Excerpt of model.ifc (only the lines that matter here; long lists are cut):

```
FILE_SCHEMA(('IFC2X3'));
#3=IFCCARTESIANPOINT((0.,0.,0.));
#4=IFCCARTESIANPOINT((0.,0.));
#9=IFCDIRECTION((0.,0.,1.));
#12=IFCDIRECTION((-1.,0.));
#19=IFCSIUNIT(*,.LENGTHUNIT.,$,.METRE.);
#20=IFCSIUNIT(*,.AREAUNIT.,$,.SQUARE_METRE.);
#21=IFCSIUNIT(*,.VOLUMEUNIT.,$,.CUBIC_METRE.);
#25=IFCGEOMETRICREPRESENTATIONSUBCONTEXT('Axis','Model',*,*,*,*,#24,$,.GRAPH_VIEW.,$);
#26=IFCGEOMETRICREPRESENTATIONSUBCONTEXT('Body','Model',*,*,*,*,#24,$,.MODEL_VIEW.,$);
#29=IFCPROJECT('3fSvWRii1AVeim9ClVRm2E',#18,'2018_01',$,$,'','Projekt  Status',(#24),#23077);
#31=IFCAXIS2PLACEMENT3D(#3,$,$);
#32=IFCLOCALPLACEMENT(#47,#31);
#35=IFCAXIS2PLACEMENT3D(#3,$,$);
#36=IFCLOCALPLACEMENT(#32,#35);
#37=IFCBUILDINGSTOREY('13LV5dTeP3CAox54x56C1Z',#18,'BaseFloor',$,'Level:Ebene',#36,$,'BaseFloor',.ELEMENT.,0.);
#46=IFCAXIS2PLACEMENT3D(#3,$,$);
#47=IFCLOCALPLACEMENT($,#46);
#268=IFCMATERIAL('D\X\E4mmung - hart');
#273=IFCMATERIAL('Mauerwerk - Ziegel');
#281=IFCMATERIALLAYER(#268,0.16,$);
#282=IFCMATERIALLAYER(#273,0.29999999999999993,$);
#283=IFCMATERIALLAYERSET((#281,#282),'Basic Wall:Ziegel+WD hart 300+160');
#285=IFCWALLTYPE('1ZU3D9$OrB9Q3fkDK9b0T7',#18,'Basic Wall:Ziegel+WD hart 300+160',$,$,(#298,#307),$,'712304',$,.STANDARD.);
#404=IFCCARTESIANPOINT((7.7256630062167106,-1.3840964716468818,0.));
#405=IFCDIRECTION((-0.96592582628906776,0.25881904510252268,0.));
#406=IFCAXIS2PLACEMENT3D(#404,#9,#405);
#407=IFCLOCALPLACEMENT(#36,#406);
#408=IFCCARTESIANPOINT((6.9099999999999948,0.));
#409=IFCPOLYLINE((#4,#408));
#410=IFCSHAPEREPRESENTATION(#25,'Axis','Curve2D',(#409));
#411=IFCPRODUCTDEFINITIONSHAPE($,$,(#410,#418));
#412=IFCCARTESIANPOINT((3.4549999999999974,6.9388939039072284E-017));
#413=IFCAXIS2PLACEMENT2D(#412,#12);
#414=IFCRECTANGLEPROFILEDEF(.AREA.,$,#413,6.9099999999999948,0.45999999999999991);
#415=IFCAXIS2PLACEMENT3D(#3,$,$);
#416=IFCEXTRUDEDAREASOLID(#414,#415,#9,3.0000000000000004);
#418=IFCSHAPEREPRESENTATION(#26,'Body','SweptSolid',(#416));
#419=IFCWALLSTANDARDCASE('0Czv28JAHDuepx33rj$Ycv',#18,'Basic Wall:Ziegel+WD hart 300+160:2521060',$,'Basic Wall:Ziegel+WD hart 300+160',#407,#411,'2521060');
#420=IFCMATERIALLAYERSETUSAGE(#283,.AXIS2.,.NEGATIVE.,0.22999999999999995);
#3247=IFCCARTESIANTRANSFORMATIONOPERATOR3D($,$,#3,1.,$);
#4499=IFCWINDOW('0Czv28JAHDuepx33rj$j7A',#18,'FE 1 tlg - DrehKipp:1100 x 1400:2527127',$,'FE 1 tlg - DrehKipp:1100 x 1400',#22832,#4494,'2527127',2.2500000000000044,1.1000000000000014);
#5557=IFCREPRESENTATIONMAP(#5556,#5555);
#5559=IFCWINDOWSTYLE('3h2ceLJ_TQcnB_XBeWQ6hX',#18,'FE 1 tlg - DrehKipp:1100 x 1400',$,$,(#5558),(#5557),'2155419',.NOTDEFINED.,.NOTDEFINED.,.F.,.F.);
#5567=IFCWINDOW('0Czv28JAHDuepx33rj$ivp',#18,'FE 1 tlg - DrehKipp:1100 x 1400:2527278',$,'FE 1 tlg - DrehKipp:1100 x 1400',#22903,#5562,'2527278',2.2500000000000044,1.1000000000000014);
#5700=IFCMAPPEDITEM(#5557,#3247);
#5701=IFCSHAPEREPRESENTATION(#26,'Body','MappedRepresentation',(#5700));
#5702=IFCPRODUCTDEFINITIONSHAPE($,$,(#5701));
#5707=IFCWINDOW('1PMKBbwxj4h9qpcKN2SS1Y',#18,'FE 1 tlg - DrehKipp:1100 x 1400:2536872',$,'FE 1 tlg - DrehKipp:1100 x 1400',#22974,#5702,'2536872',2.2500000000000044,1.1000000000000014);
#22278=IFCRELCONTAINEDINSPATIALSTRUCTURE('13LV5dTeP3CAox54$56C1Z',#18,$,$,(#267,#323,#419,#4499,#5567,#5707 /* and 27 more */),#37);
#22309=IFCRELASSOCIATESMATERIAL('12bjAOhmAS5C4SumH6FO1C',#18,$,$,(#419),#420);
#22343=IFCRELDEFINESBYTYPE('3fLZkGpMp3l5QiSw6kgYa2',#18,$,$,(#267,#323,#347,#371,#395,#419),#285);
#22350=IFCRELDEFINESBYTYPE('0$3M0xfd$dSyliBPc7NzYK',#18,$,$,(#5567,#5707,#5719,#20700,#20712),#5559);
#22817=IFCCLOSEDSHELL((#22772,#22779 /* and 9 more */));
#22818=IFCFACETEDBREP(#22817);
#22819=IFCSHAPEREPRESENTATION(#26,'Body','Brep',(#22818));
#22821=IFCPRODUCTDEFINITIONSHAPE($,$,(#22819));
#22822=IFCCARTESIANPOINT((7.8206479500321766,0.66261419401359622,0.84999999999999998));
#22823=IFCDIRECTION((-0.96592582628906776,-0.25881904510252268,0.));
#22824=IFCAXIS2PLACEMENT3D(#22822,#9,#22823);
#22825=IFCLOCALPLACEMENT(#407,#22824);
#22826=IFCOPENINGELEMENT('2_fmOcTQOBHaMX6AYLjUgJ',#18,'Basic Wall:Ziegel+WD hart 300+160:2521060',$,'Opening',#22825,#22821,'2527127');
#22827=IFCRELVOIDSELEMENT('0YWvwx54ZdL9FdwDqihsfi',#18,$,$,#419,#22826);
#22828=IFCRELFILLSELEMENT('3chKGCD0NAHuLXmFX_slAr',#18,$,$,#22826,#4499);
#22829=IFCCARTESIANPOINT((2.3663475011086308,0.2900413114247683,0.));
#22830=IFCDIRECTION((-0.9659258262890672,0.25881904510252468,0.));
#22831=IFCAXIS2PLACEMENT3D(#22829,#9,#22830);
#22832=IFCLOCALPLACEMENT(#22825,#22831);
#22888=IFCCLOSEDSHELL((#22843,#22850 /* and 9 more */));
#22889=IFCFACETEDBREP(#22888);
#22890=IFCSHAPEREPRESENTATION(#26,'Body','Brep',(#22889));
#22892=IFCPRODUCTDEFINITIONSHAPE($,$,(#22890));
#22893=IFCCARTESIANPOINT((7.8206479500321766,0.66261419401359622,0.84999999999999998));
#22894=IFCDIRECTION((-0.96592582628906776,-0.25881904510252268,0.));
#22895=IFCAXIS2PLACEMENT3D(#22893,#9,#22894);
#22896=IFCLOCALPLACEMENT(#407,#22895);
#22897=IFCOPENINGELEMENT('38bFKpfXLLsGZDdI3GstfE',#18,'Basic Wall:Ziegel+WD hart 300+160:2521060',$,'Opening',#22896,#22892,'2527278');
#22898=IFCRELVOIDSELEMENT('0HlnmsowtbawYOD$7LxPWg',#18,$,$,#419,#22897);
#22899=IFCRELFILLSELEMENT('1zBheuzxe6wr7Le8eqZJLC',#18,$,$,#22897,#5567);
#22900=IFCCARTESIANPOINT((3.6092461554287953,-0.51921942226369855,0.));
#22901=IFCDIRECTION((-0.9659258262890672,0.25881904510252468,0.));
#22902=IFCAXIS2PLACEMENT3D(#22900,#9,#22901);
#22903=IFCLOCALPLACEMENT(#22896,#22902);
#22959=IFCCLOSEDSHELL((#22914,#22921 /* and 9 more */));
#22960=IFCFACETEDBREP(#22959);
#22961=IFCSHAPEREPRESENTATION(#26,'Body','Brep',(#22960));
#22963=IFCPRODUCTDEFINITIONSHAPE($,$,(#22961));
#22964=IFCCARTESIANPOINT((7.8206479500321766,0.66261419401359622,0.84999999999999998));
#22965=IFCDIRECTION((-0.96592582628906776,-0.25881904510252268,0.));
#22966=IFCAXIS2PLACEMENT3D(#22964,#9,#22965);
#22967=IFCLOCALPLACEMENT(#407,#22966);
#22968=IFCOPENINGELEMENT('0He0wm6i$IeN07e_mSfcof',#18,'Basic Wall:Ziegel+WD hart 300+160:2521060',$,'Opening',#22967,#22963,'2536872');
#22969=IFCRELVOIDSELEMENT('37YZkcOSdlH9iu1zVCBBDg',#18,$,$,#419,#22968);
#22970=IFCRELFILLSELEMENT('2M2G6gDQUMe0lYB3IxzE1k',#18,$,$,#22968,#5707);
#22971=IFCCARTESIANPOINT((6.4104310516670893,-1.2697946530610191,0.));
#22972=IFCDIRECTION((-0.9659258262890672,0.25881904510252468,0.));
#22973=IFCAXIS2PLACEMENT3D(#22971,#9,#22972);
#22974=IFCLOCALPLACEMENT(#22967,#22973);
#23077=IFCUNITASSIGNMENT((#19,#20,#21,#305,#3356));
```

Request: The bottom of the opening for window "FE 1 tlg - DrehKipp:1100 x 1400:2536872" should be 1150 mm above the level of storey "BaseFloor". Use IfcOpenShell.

```python
import numpy as np
import ifcopenshell
import ifcopenshell.api.geometry
import ifcopenshell.geom
import ifcopenshell.util.element
import ifcopenshell.util.placement
import ifcopenshell.util.shape
import ifcopenshell.util.unit

model = ifcopenshell.open("model.ifc")
unit_scale = ifcopenshell.util.unit.calculate_unit_scale(model)

window = model.by_guid("1PMKBbwxj4h9qpcKN2SS1Y")
opening = window.FillsVoids[0].RelatingOpeningElement
storey = ifcopenshell.util.element.get_container(window, ifc_class="IfcBuildingStorey")
level = ifcopenshell.util.placement.get_local_placement(storey.ObjectPlacement)[2, 3]

# The opening's origin need not be at the sill, so measure its lowest point.
shape = ifcopenshell.geom.create_shape(ifcopenshell.geom.settings(), opening)
bottom = ifcopenshell.util.shape.get_shape_bottom_elevation(shape, shape.geometry) / unit_scale
dz = level + 1.15 - bottom

shift = np.array([0.0, 0.0, dz])
# The window is placed relative to its opening, so it follows when the opening moves.
matrix = ifcopenshell.util.placement.get_local_placement(opening.ObjectPlacement)
matrix[:3, 3] += shift
ifcopenshell.api.geometry.edit_object_placement(
    model, product=opening, matrix=matrix, is_si=False, should_transform_children=True
)

print(f"moved by {dz * unit_scale:+.3f} m")

model.write("model_edited.ifc")
```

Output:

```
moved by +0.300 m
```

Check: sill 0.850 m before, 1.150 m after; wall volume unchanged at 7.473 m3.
